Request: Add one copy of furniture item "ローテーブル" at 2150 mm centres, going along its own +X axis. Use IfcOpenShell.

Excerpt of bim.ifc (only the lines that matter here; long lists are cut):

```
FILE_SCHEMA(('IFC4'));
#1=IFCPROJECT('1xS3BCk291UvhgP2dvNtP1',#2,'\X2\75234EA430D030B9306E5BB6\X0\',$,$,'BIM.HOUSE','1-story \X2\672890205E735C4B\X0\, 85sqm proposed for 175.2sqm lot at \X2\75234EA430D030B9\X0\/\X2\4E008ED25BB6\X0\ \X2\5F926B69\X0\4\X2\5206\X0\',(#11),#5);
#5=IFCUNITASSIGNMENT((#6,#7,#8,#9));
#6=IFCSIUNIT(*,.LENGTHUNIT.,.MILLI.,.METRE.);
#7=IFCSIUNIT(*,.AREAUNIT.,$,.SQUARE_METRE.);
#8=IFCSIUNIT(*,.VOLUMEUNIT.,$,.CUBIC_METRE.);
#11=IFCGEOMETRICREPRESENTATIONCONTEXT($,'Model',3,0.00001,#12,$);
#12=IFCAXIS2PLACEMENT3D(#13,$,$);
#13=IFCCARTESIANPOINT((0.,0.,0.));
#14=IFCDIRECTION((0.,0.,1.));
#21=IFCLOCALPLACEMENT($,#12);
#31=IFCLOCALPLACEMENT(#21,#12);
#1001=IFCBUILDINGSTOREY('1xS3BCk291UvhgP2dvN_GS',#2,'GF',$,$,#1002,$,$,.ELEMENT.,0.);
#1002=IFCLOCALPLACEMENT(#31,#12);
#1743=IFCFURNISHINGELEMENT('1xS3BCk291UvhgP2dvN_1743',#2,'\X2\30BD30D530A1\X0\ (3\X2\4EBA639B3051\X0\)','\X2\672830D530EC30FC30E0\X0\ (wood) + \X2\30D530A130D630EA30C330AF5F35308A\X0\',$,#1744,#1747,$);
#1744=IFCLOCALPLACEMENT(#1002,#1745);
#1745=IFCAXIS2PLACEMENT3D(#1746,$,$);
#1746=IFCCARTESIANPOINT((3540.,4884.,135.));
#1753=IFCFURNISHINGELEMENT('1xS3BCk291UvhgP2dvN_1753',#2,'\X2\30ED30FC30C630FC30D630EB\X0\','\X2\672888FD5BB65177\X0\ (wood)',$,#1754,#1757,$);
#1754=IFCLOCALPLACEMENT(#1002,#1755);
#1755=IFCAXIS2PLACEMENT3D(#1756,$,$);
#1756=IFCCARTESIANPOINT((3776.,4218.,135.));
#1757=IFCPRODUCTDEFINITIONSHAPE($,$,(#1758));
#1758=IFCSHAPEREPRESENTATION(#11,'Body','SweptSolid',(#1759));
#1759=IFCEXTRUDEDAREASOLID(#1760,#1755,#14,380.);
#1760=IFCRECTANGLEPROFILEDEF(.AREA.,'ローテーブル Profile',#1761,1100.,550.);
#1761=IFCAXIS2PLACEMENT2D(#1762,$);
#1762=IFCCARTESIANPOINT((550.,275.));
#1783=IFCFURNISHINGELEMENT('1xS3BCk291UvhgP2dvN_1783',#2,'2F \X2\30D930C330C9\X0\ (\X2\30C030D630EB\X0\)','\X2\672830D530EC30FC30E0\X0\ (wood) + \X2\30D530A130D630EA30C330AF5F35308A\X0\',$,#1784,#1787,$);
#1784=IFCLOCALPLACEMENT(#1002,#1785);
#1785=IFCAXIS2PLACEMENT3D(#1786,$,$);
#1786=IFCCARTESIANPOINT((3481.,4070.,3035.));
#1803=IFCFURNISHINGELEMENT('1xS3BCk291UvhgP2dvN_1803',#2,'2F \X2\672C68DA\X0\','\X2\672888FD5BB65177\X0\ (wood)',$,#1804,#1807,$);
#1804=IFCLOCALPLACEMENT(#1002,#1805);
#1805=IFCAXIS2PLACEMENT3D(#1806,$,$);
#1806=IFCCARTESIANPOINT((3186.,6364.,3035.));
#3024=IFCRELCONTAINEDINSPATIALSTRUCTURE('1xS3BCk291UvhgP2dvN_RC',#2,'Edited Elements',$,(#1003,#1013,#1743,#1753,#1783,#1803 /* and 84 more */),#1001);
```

```python
import ifcopenshell
import ifcopenshell.api.geometry
import ifcopenshell.api.root
import ifcopenshell.util.element
import ifcopenshell.util.placement

model = ifcopenshell.open("bim.ifc")


def reuse_history(source, copy):
    """copy_class also copies each property set's owner history, people and application; keep the originals."""
    for rel in copy.IsDefinedBy:
        if rel.is_a("IfcRelDefinesByProperties") and (history := rel.RelatingPropertyDefinition.OwnerHistory):
            rel.RelatingPropertyDefinition.OwnerHistory = source.OwnerHistory
            ifcopenshell.util.element.remove_deep2(model, history)


source = model.by_guid("1xS3BCk291UvhgP2dvN_1753")
base = ifcopenshell.util.placement.get_local_placement(source.ObjectPlacement)
step = base[:3, 0] * 2150.0

for i in range(1, 2):
    copy = ifcopenshell.api.root.copy_class(model, product=source)
    copy.Representation = ifcopenshell.util.element.copy_deep(
        model, source.Representation, exclude=["IfcGeometricRepresentationContext", "IfcRepresentationMap"]
    )
    reuse_history(source, copy)
    matrix = base.copy()
    matrix[:3, 3] += i * step
    print("added at", matrix[:3, 3].round(3) + 0.0)
    ifcopenshell.api.geometry.edit_object_placement(model, product=copy, matrix=matrix, is_si=False)

model.write("bim_edited.ifc")
```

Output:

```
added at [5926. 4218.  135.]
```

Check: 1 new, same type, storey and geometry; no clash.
